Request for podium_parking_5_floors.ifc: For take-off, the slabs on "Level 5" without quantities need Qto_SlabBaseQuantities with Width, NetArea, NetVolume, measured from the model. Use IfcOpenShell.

First a look at what the model holds.

```python
import ifcopenshell
import ifcopenshell.util.element
import ifcopenshell.util.unit

model = ifcopenshell.open("podium_parking_5_floors.ifc")
print(model.schema)
for unit_type in ("LENGTHUNIT", "AREAUNIT", "VOLUMEUNIT"):
    print(unit_type, ifcopenshell.util.unit.calculate_unit_scale(model, unit_type))
storey = next(s for s in model.by_type("IfcBuildingStorey") if s.Name == "Level 5")
slabs = [e for e in ifcopenshell.util.element.get_decomposition(storey) if e.is_a("IfcSlab")]
for e in sorted(slabs, key=lambda e: e.id()):
    print(e.id(), e.is_a(), e.Name, list(ifcopenshell.util.element.get_psets(e, qtos_only=True)), sep=" | ")
```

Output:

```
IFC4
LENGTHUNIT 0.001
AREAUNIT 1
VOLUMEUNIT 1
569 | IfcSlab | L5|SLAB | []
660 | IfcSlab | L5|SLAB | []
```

```python
import ifcopenshell
import ifcopenshell.api.pset
import ifcopenshell.geom
import ifcopenshell.util.element
import ifcopenshell.util.shape
import ifcopenshell.util.unit

model = ifcopenshell.open("podium_parking_5_floors.ifc")
unit_scale = ifcopenshell.util.unit.calculate_unit_scale(model)
area_scale = ifcopenshell.util.unit.calculate_unit_scale(model, "AREAUNIT")
volume_scale = ifcopenshell.util.unit.calculate_unit_scale(model, "VOLUMEUNIT")
settings = ifcopenshell.geom.settings()

storey = next(s for s in model.by_type("IfcBuildingStorey") if s.Name == "Level 5")
slabs = [e for e in ifcopenshell.util.element.get_decomposition(storey) if e.is_a("IfcSlab")]

for e in sorted(slabs, key=lambda e: e.id()):
    if ifcopenshell.util.element.get_psets(e, qtos_only=True, should_inherit=False):
        continue
    # Geometry comes back in metres, in the element's own axes.
    shape = ifcopenshell.geom.create_shape(settings, e)
    values = {
        "Width": ifcopenshell.util.shape.get_z(shape.geometry) / unit_scale,
        "NetArea": ifcopenshell.util.shape.get_footprint_area(shape.geometry) / area_scale,
        "NetVolume": ifcopenshell.util.shape.get_volume(shape.geometry) / volume_scale,
    }
    qto = ifcopenshell.api.pset.add_qto(model, product=e, name="Qto_SlabBaseQuantities")
    ifcopenshell.api.pset.edit_qto(model, qto=qto, properties=values)
    print(e.id(), {k: round(v, 3) for k, v in values.items()})

model.write("podium_parking_5_floors-out.ifc")
```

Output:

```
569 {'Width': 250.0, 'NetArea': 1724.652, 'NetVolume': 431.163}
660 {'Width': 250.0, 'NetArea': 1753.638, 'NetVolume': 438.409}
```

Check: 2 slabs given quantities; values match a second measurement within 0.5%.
